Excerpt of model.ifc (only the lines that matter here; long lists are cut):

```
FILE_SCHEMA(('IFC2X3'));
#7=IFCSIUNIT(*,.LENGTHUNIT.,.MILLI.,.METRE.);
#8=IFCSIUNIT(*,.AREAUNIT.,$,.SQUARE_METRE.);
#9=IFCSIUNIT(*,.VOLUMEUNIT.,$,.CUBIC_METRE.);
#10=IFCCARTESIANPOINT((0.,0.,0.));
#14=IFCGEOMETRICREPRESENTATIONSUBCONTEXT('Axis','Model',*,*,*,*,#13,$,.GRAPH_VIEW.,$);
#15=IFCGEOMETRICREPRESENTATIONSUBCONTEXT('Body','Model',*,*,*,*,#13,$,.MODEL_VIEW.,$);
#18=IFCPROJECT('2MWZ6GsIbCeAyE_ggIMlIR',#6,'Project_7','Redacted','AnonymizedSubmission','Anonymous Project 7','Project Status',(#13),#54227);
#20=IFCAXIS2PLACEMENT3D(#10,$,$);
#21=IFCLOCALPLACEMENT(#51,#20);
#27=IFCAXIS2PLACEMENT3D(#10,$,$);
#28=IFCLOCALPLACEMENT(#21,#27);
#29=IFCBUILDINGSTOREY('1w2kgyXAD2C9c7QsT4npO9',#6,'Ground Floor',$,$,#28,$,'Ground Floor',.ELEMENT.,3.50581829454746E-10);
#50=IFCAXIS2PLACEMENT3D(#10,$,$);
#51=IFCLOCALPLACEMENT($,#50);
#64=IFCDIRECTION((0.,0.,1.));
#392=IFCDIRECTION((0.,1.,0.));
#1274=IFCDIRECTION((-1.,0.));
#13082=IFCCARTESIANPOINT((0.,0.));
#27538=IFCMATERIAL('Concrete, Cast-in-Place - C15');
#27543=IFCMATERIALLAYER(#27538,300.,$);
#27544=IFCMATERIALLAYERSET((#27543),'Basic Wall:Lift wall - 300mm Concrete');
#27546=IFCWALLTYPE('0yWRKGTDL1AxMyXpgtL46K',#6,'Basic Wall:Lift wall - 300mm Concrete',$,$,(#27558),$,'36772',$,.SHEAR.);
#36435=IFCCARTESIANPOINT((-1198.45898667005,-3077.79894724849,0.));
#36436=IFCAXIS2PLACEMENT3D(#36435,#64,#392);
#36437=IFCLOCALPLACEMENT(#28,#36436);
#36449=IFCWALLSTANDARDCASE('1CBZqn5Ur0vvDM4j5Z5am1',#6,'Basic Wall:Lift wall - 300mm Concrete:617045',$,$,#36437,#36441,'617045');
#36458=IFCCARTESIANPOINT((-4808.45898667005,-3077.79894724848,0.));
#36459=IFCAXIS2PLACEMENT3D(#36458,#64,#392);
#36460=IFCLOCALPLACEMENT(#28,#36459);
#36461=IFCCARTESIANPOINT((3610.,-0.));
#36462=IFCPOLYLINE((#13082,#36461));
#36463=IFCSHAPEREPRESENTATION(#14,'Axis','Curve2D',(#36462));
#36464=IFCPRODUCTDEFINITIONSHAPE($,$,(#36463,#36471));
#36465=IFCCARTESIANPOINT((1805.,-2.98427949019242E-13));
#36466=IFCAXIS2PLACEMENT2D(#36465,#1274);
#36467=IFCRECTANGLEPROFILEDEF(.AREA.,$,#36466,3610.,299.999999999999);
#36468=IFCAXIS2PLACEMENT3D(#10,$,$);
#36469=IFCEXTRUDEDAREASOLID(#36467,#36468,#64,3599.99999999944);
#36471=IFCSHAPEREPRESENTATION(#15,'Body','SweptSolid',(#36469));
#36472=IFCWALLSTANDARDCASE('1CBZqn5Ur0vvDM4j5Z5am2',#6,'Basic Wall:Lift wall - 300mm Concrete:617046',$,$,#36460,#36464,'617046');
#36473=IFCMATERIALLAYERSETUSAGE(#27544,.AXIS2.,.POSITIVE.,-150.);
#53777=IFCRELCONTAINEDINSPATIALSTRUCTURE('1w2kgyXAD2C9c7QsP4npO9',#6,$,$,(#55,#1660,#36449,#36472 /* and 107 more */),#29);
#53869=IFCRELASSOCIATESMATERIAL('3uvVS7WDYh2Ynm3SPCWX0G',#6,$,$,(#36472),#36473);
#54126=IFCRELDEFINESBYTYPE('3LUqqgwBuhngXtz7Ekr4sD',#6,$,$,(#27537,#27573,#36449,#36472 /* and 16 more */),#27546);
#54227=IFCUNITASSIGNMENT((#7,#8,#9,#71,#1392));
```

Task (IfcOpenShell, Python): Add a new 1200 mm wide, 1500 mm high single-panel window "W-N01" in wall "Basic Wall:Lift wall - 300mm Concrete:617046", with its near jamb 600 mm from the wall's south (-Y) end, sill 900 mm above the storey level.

```python
import numpy as np
import ifcopenshell
import ifcopenshell.api.feature
import ifcopenshell.api.geometry
import ifcopenshell.api.root
import ifcopenshell.api.spatial
import ifcopenshell.api.type
import ifcopenshell.geom
import ifcopenshell.util.element
import ifcopenshell.util.placement
import ifcopenshell.util.representation
import ifcopenshell.util.shape
import ifcopenshell.util.unit

model = ifcopenshell.open("model.ifc")
unit_scale = ifcopenshell.util.unit.calculate_unit_scale(model)
settings = ifcopenshell.geom.settings()


def volume(element):
    """Net volume in cubic metres, openings subtracted."""
    shape = ifcopenshell.geom.create_shape(settings, element)
    return ifcopenshell.util.shape.get_volume(shape.geometry)


wall = model.by_id(36472)
storey = ifcopenshell.util.element.get_container(wall, ifc_class="IfcBuildingStorey")
context = ifcopenshell.util.representation.get_context(model, "Model", "Body", "MODEL_VIEW")
before = volume(wall)

width, height, from_end, sill = 1.2, 1.5, 0.6, 0.9  # metres

# The wall runs along its own X axis, and the end named is its -X end.
wall_shape = ifcopenshell.geom.create_shape(settings, wall)
x, y, z = ifcopenshell.util.shape.get_vertices(wall_shape.geometry).T
start = x.min() + from_end
face, thickness = float(y.min()), float(y.max() - y.min())
wall_matrix = ifcopenshell.util.placement.get_local_placement(wall.ObjectPlacement)
level = ifcopenshell.util.placement.get_local_placement(storey.ObjectPlacement)[2, 3]


def in_wall(x, y):
    """Placement at x, y metres in the wall's axes, at sill height."""
    matrix = wall_matrix.copy()
    matrix[:, 3] = wall_matrix @ np.array([x / unit_scale, y / unit_scale, 0.0, 1.0])
    matrix[2, 3] = level + sill / unit_scale
    return matrix


# Opening: a box that overshoots both wall faces by 50 mm.
opening = ifcopenshell.api.root.create_entity(model, ifc_class="IfcOpeningElement")
box = ifcopenshell.api.geometry.add_wall_representation(
    model, context=context, length=width, height=height, thickness=thickness + 0.1
)
ifcopenshell.api.geometry.assign_representation(model, product=opening, representation=box)
ifcopenshell.api.geometry.edit_object_placement(model, product=opening, matrix=in_wall(start, face - 0.05), is_si=False)
ifcopenshell.api.feature.add_feature(model, feature=opening, element=wall)

window = ifcopenshell.api.root.create_entity(model, ifc_class="IfcWindow", name="W-N01")
window.OverallWidth, window.OverallHeight = width / unit_scale, height / unit_scale
body = ifcopenshell.api.geometry.add_window_representation(
    model,
    context=context,
    overall_width=window.OverallWidth,
    overall_height=window.OverallHeight,
    partition_type="SINGLE_PANEL",
)
ifcopenshell.api.geometry.assign_representation(model, product=window, representation=body)
ifcopenshell.api.spatial.assign_container(model, products=[window], relating_structure=storey)
fills = ifcopenshell.api.feature.add_filling(model, opening=opening, element=window)
fills.OwnerHistory = window.OwnerHistory  # required in IFC2X3

# IFC2X3 keeps the operation on the window style.
style = ifcopenshell.api.root.create_entity(model, ifc_class="IfcWindowStyle", name="W-N01")
style.OperationType, style.ConstructionType = "SINGLE_PANEL", "NOTDEFINED"
style.ParameterTakesPrecedence = style.Sizeable = False
ifcopenshell.api.type.assign_type(model, related_objects=[window], relating_type=style)

# Centre the window in the wall's thickness.
ifcopenshell.api.geometry.edit_object_placement(model, product=window, matrix=in_wall(start, face), is_si=False)
window_shape = ifcopenshell.geom.create_shape(settings, window)
depth = ifcopenshell.util.shape.get_vertices(window_shape.geometry)[:, 1]
offset = face + thickness / 2 - (depth.min() + depth.max()) / 2
ifcopenshell.api.geometry.edit_object_placement(model, product=window, matrix=in_wall(start, offset), is_si=False)

after = volume(wall)

print(f"wall volume {before:.3f} -> {after:.3f} m3")

model.write("model_edited.ifc")
```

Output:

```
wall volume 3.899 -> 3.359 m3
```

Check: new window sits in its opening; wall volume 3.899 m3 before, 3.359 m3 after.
